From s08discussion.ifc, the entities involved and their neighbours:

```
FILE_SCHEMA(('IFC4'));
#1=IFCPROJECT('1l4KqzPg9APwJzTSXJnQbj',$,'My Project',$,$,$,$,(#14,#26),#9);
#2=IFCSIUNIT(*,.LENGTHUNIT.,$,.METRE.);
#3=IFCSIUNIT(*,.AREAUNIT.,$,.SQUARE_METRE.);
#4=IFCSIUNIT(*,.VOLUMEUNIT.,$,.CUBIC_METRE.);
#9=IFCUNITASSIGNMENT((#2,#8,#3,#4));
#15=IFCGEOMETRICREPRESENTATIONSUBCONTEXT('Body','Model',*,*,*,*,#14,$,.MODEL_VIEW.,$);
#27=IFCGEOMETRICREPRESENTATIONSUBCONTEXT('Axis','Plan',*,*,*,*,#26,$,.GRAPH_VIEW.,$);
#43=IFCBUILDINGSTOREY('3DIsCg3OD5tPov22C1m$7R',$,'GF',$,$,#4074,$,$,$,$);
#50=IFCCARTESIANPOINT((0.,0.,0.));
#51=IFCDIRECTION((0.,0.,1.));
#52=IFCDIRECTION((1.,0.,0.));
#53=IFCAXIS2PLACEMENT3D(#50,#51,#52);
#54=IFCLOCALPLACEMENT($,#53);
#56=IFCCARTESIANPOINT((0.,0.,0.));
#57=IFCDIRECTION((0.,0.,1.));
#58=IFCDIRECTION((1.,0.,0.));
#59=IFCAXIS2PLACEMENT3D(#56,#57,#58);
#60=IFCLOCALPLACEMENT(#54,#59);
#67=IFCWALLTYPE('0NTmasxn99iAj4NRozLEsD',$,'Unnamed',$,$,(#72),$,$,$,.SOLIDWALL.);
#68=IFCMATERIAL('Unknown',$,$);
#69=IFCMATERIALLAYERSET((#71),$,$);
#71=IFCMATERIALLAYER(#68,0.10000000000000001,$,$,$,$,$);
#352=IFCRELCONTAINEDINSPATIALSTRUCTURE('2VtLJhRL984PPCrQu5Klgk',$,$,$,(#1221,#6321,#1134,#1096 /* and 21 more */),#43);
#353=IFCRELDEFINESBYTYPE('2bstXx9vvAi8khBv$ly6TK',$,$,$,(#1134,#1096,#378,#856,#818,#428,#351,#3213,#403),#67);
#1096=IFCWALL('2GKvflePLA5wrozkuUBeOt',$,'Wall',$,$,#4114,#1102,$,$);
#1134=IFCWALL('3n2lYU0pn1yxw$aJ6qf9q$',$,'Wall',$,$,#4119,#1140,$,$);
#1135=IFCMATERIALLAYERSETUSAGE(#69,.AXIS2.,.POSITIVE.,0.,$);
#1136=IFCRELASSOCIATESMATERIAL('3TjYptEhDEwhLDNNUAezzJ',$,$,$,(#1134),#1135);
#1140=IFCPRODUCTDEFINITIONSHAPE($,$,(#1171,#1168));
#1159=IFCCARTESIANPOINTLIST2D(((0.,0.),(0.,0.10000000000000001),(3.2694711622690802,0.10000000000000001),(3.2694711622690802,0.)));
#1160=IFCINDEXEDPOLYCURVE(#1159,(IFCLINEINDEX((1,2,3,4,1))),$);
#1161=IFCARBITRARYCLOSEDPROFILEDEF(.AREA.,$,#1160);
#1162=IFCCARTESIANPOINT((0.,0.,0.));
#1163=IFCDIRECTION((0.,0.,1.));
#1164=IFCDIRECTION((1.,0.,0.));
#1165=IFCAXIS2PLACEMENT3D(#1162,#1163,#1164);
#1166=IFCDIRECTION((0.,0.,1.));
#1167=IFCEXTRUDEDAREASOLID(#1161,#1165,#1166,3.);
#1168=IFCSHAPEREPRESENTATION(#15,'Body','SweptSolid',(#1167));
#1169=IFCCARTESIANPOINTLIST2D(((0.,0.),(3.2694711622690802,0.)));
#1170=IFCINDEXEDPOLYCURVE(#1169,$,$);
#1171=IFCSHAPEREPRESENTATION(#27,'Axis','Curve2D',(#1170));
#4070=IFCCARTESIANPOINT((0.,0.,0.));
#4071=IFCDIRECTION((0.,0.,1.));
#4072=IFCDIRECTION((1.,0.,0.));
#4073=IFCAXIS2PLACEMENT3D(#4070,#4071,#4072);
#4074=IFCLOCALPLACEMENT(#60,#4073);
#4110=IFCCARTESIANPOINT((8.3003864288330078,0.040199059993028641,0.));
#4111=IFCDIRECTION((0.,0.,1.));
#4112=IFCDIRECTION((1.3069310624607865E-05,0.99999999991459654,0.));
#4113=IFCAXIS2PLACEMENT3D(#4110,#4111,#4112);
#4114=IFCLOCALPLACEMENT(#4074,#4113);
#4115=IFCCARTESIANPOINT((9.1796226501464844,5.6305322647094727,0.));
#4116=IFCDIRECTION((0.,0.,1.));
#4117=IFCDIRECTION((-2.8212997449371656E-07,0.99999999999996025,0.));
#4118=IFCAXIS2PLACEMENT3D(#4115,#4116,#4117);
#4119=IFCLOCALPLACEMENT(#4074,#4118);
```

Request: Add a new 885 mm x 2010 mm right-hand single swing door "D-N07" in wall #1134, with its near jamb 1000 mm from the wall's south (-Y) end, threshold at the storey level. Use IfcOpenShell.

```python
import numpy as np
import ifcopenshell
import ifcopenshell.api.feature
import ifcopenshell.api.geometry
import ifcopenshell.api.root
import ifcopenshell.api.spatial
import ifcopenshell.geom
import ifcopenshell.util.element
import ifcopenshell.util.placement
import ifcopenshell.util.representation
import ifcopenshell.util.shape
import ifcopenshell.util.unit

model = ifcopenshell.open("s08discussion.ifc")
unit_scale = ifcopenshell.util.unit.calculate_unit_scale(model)
settings = ifcopenshell.geom.settings()


def volume(element):
    """Net volume in cubic metres, openings subtracted."""
    shape = ifcopenshell.geom.create_shape(settings, element)
    return ifcopenshell.util.shape.get_volume(shape.geometry)


wall = model.by_id(1134)
storey = ifcopenshell.util.element.get_container(wall, ifc_class="IfcBuildingStorey")
context = ifcopenshell.util.representation.get_context(model, "Model", "Body", "MODEL_VIEW")
before = volume(wall)

width, height, from_end, sill = 0.885, 2.01, 1, 0.0  # metres

# The wall runs along its own X axis, and the end named is its -X end.
wall_shape = ifcopenshell.geom.create_shape(settings, wall)
x, y, z = ifcopenshell.util.shape.get_vertices(wall_shape.geometry).T
start = x.min() + from_end
face, thickness = float(y.min()), float(y.max() - y.min())
wall_matrix = ifcopenshell.util.placement.get_local_placement(wall.ObjectPlacement)
level = ifcopenshell.util.placement.get_local_placement(storey.ObjectPlacement)[2, 3]


def in_wall(x, y):
    """Placement at x, y metres in the wall's axes, at sill height."""
    matrix = wall_matrix.copy()
    matrix[:, 3] = wall_matrix @ np.array([x / unit_scale, y / unit_scale, 0.0, 1.0])
    matrix[2, 3] = level + sill / unit_scale
    return matrix


# Opening: a box that overshoots both wall faces by 50 mm.
opening = ifcopenshell.api.root.create_entity(model, ifc_class="IfcOpeningElement", predefined_type="OPENING")
box = ifcopenshell.api.geometry.add_wall_representation(
    model, context=context, length=width, height=height, thickness=thickness + 0.1
)
ifcopenshell.api.geometry.assign_representation(model, product=opening, representation=box)
ifcopenshell.api.geometry.edit_object_placement(model, product=opening, matrix=in_wall(start, face - 0.05), is_si=False)
ifcopenshell.api.feature.add_feature(model, feature=opening, element=wall)

door = ifcopenshell.api.root.create_entity(model, ifc_class="IfcDoor", name="D-N07", predefined_type="DOOR")
door.OverallWidth, door.OverallHeight = width / unit_scale, height / unit_scale
door.OperationType = "SINGLE_SWING_RIGHT"
body = ifcopenshell.api.geometry.add_door_representation(
    model,
    context=context,
    overall_width=door.OverallWidth,
    overall_height=door.OverallHeight,
    operation_type="SINGLE_SWING_RIGHT",
    lining_properties={"LiningDepth": thickness / unit_scale, "ThresholdDepth": thickness / unit_scale},
)
ifcopenshell.api.geometry.assign_representation(model, product=door, representation=body)
ifcopenshell.api.spatial.assign_container(model, products=[door], relating_structure=storey)
ifcopenshell.api.feature.add_filling(model, opening=opening, element=door)

# The lining spans the wall, so the door starts at the wall face.
ifcopenshell.api.geometry.edit_object_placement(model, product=door, matrix=in_wall(start, face), is_si=False)

after = volume(wall)

print(f"wall volume {before:.3f} -> {after:.3f} m3")

model.write("s08discussion_rev.ifc")
```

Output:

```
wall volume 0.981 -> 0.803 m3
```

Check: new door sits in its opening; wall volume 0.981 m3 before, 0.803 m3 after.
